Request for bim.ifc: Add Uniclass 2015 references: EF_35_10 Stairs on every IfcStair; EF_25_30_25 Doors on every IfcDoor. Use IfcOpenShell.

First a look at what the model holds.

```python
import ifcopenshell

model = ifcopenshell.open("bim.ifc")
print(model.schema)
print("classifications:", [c.Name for c in model.by_type("IfcClassification")])
for ifc_class in ("IfcDoor", "IfcRoof", "IfcStair", "IfcWall", "IfcWindow"):
    print(ifc_class, len(model.by_type(ifc_class)))
```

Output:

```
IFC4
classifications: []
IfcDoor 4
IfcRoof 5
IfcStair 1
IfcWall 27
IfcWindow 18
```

```python
import ifcopenshell
import ifcopenshell.api.classification

model = ifcopenshell.open("bim.ifc")

system = ifcopenshell.api.classification.add_classification(model, classification="Uniclass 2015")

codes = {
    "IfcStair": ("EF_35_10", "Stairs"),
    "IfcDoor": ("EF_25_30_25", "Doors"),
}
for ifc_class, (code, name) in codes.items():
    products = model.by_type(ifc_class)
    ifcopenshell.api.classification.add_reference(
        model, products=products, classification=system, identification=code, name=name
    )
    print(code, len(products))

model.write("bim_edited.ifc")
```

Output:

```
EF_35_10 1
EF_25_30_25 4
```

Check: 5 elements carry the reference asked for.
